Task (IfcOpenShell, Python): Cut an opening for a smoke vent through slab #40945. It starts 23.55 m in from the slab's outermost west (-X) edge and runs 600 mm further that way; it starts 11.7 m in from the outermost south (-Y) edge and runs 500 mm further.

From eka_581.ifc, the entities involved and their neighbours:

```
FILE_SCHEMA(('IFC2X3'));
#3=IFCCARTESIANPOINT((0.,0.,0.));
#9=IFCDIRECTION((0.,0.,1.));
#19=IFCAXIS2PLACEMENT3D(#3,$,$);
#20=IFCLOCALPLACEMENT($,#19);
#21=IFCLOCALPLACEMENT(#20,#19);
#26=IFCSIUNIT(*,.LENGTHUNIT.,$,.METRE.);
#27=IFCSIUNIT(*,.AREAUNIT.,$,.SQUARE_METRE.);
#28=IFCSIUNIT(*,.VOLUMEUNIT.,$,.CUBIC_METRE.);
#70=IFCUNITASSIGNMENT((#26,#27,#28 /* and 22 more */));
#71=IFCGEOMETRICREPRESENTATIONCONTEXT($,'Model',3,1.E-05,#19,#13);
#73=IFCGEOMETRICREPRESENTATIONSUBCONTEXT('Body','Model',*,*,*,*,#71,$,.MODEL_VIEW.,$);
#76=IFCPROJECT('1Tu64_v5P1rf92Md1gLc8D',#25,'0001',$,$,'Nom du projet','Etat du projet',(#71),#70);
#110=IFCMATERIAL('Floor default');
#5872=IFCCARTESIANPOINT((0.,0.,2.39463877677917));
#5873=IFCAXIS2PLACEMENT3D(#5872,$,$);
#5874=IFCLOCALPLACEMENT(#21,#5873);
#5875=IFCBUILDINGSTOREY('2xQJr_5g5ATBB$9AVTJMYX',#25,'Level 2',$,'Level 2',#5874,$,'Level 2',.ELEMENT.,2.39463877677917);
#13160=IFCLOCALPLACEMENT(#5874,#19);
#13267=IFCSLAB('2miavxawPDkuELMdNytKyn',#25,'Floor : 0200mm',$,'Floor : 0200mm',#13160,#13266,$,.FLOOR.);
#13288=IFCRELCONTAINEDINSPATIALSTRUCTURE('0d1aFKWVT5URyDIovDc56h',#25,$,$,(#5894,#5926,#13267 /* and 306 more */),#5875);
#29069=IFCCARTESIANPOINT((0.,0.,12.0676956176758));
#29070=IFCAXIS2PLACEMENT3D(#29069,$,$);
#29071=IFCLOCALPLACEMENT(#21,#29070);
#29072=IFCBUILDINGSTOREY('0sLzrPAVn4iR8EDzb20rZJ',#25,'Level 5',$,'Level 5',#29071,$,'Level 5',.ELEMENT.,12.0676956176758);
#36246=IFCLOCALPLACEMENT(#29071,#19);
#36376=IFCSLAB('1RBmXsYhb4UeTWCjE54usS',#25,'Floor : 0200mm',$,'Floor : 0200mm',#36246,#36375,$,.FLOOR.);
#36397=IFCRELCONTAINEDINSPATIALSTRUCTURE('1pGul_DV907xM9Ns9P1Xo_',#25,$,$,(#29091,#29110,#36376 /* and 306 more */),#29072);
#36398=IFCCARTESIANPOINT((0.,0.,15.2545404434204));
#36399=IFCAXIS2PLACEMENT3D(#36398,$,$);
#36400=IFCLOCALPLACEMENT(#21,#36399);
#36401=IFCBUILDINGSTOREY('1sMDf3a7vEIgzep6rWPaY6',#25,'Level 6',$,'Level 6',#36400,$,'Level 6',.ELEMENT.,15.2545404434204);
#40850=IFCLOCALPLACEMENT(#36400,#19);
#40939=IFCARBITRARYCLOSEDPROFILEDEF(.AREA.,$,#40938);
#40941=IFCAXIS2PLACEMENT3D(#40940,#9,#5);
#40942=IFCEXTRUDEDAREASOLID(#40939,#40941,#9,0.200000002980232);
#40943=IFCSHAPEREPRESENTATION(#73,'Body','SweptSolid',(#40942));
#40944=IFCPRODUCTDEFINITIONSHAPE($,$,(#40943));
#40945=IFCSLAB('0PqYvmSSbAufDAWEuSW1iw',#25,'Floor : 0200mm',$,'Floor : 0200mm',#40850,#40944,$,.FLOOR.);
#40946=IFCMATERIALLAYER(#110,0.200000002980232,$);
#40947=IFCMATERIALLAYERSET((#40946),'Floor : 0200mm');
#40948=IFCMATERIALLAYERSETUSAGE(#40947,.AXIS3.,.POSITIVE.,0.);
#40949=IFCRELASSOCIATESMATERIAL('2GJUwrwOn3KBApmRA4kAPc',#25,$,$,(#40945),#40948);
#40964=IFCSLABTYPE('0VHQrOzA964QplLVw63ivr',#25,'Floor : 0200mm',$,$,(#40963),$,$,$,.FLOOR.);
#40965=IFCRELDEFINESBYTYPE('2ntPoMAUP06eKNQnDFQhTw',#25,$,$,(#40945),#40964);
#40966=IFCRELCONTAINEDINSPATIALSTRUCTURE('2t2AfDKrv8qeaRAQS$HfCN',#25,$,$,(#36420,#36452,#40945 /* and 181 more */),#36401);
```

```python
import numpy as np
import ifcopenshell
import ifcopenshell.api.feature
import ifcopenshell.api.geometry
import ifcopenshell.api.root
import ifcopenshell.geom
import ifcopenshell.util.placement
import ifcopenshell.util.representation
import ifcopenshell.util.shape
import ifcopenshell.util.unit

model = ifcopenshell.open("eka_581.ifc")
unit_scale = ifcopenshell.util.unit.calculate_unit_scale(model)
settings = ifcopenshell.geom.settings()


def volume(element):
    """Net volume in cubic metres, openings subtracted."""
    shape = ifcopenshell.geom.create_shape(settings, element)
    return ifcopenshell.util.shape.get_volume(shape.geometry)


slab = model.by_guid("0PqYvmSSbAufDAWEuSW1iw")
before = volume(slab)

# Extent in the slab's own axes, in metres. The edges named are its -X and -Y sides.
slab_shape = ifcopenshell.geom.create_shape(settings, slab)
vertices = ifcopenshell.util.shape.get_vertices(slab_shape.geometry)
x_min, y_min, bottom = vertices.min(axis=0)
top = vertices[:, 2].max()

opening = ifcopenshell.api.root.create_entity(model, ifc_class="IfcOpeningElement", name="Smoke vent opening")
context = ifcopenshell.util.representation.get_context(model, "Model", "Body", "MODEL_VIEW")
width, depth = 0.6, 0.5
outline = [(0.0, 0.0), (width, 0.0), (width, depth), (0.0, depth), (0.0, 0.0)]
# Overshoot both faces by 50 mm so the cut is clean.
shape = ifcopenshell.api.geometry.add_slab_representation(
    model, context=context, depth=top - bottom + 0.1, polyline=outline
)
ifcopenshell.api.geometry.assign_representation(model, product=opening, representation=shape)

matrix = ifcopenshell.util.placement.get_local_placement(slab.ObjectPlacement)
matrix[:, 3] = matrix @ np.append(np.array([x_min + 23.55, y_min + 11.7, bottom - 0.05]) / unit_scale, 1.0)
ifcopenshell.api.geometry.edit_object_placement(model, product=opening, matrix=matrix, is_si=False)
ifcopenshell.api.feature.add_feature(model, feature=opening, element=slab)

after = volume(slab)

print(f"slab volume {before:.3f} -> {after:.3f} m3")

model.write("eka_581_edited.ifc")
```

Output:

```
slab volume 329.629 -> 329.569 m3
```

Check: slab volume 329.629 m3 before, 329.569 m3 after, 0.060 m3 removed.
